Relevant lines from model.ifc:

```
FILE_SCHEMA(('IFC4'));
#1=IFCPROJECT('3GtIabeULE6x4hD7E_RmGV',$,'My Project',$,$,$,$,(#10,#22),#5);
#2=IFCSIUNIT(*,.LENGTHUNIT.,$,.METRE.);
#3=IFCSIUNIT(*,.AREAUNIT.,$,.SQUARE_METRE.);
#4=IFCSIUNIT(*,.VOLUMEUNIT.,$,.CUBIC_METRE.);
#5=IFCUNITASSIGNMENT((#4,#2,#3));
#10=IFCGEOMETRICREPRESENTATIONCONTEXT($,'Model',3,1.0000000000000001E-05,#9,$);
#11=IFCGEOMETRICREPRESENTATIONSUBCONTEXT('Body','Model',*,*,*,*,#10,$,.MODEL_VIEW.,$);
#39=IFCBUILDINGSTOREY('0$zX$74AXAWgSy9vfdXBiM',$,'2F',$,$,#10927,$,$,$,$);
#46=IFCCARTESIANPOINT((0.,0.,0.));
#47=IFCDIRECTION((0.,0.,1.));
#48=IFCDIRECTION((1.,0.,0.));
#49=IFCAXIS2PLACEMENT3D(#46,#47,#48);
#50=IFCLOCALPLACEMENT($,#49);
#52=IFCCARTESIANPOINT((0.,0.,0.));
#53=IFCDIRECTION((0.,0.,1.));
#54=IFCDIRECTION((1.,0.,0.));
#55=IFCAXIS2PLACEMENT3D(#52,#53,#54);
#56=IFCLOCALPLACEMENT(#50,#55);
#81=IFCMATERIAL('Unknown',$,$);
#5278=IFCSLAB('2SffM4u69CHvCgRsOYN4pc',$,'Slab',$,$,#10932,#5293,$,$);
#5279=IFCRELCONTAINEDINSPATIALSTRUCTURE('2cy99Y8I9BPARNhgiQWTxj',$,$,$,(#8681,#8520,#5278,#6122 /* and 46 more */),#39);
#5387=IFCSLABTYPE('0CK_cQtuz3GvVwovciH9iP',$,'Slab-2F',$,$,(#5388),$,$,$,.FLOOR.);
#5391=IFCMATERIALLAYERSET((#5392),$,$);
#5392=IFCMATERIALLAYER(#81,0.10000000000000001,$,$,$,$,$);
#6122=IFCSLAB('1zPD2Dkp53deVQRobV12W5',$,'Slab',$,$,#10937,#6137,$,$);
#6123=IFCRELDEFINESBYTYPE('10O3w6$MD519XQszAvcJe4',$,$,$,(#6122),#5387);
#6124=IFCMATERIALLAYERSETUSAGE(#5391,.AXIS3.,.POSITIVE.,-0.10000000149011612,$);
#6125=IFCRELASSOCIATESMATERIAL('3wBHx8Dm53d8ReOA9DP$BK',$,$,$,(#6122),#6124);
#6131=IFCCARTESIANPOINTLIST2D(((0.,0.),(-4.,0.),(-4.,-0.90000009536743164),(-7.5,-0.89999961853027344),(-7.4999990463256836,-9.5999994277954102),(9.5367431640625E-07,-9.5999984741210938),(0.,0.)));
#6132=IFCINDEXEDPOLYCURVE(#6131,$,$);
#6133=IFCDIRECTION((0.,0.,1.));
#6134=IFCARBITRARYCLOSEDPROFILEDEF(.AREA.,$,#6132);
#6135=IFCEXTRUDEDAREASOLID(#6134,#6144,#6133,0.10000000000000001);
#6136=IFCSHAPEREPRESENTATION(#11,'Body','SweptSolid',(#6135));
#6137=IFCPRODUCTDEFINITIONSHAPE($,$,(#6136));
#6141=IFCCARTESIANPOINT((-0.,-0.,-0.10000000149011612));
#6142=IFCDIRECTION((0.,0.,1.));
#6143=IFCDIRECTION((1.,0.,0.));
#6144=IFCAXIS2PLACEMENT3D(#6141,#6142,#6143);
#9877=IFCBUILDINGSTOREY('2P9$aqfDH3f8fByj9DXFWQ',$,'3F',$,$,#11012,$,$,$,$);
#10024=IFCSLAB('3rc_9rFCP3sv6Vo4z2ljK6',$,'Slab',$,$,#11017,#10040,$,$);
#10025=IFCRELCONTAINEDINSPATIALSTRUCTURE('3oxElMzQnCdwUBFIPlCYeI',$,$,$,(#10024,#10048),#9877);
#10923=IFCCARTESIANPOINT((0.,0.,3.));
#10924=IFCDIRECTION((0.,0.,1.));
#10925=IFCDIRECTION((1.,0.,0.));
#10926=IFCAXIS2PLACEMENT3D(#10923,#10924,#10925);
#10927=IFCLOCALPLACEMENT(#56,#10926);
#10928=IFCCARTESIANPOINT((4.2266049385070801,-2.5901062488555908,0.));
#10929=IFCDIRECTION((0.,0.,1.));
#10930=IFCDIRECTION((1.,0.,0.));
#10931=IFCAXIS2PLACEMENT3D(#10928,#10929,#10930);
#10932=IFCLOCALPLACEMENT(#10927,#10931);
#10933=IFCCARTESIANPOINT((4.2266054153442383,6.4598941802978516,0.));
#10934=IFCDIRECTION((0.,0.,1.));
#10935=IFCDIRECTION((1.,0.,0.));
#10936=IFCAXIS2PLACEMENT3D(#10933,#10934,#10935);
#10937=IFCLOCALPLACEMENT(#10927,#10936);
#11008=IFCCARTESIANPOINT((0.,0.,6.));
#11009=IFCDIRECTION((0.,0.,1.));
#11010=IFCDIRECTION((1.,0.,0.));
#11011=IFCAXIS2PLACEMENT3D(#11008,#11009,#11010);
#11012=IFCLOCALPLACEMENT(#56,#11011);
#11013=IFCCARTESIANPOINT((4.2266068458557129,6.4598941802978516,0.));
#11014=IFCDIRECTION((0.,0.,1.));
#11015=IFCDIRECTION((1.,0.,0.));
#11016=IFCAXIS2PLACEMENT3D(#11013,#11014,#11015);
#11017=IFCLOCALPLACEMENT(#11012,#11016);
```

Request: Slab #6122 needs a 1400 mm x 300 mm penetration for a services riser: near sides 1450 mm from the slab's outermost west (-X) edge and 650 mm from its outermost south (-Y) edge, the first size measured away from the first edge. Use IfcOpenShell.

```python
import numpy as np
import ifcopenshell
import ifcopenshell.api.feature
import ifcopenshell.api.geometry
import ifcopenshell.api.root
import ifcopenshell.geom
import ifcopenshell.util.placement
import ifcopenshell.util.representation
import ifcopenshell.util.shape
import ifcopenshell.util.unit

model = ifcopenshell.open("model.ifc")
unit_scale = ifcopenshell.util.unit.calculate_unit_scale(model)
settings = ifcopenshell.geom.settings()


def volume(element):
    """Net volume in cubic metres, openings subtracted."""
    shape = ifcopenshell.geom.create_shape(settings, element)
    return ifcopenshell.util.shape.get_volume(shape.geometry)


slab = model.by_guid("1zPD2Dkp53deVQRobV12W5")
before = volume(slab)

# Extent in the slab's own axes, in metres. The edges named are its -X and -Y sides.
slab_shape = ifcopenshell.geom.create_shape(settings, slab)
vertices = ifcopenshell.util.shape.get_vertices(slab_shape.geometry)
x_min, y_min, bottom = vertices.min(axis=0)
top = vertices[:, 2].max()

opening = ifcopenshell.api.root.create_entity(model, ifc_class="IfcOpeningElement", name="Services riser opening", predefined_type="OPENING")
context = ifcopenshell.util.representation.get_context(model, "Model", "Body", "MODEL_VIEW")
width, depth = 1.4, 0.3
outline = [(0.0, 0.0), (width, 0.0), (width, depth), (0.0, depth), (0.0, 0.0)]
# Overshoot both faces by 50 mm so the cut is clean.
shape = ifcopenshell.api.geometry.add_slab_representation(
    model, context=context, depth=top - bottom + 0.1, polyline=outline
)
ifcopenshell.api.geometry.assign_representation(model, product=opening, representation=shape)

matrix = ifcopenshell.util.placement.get_local_placement(slab.ObjectPlacement)
matrix[:, 3] = matrix @ np.append(np.array([x_min + 1.45, y_min + 0.65, bottom - 0.05]) / unit_scale, 1.0)
ifcopenshell.api.geometry.edit_object_placement(model, product=opening, matrix=matrix, is_si=False)
ifcopenshell.api.feature.add_feature(model, feature=opening, element=slab)

after = volume(slab)

print(f"slab volume {before:.3f} -> {after:.3f} m3")

model.write("model_rev.ifc")
```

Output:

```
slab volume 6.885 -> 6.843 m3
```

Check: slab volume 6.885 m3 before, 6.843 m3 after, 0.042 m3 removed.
